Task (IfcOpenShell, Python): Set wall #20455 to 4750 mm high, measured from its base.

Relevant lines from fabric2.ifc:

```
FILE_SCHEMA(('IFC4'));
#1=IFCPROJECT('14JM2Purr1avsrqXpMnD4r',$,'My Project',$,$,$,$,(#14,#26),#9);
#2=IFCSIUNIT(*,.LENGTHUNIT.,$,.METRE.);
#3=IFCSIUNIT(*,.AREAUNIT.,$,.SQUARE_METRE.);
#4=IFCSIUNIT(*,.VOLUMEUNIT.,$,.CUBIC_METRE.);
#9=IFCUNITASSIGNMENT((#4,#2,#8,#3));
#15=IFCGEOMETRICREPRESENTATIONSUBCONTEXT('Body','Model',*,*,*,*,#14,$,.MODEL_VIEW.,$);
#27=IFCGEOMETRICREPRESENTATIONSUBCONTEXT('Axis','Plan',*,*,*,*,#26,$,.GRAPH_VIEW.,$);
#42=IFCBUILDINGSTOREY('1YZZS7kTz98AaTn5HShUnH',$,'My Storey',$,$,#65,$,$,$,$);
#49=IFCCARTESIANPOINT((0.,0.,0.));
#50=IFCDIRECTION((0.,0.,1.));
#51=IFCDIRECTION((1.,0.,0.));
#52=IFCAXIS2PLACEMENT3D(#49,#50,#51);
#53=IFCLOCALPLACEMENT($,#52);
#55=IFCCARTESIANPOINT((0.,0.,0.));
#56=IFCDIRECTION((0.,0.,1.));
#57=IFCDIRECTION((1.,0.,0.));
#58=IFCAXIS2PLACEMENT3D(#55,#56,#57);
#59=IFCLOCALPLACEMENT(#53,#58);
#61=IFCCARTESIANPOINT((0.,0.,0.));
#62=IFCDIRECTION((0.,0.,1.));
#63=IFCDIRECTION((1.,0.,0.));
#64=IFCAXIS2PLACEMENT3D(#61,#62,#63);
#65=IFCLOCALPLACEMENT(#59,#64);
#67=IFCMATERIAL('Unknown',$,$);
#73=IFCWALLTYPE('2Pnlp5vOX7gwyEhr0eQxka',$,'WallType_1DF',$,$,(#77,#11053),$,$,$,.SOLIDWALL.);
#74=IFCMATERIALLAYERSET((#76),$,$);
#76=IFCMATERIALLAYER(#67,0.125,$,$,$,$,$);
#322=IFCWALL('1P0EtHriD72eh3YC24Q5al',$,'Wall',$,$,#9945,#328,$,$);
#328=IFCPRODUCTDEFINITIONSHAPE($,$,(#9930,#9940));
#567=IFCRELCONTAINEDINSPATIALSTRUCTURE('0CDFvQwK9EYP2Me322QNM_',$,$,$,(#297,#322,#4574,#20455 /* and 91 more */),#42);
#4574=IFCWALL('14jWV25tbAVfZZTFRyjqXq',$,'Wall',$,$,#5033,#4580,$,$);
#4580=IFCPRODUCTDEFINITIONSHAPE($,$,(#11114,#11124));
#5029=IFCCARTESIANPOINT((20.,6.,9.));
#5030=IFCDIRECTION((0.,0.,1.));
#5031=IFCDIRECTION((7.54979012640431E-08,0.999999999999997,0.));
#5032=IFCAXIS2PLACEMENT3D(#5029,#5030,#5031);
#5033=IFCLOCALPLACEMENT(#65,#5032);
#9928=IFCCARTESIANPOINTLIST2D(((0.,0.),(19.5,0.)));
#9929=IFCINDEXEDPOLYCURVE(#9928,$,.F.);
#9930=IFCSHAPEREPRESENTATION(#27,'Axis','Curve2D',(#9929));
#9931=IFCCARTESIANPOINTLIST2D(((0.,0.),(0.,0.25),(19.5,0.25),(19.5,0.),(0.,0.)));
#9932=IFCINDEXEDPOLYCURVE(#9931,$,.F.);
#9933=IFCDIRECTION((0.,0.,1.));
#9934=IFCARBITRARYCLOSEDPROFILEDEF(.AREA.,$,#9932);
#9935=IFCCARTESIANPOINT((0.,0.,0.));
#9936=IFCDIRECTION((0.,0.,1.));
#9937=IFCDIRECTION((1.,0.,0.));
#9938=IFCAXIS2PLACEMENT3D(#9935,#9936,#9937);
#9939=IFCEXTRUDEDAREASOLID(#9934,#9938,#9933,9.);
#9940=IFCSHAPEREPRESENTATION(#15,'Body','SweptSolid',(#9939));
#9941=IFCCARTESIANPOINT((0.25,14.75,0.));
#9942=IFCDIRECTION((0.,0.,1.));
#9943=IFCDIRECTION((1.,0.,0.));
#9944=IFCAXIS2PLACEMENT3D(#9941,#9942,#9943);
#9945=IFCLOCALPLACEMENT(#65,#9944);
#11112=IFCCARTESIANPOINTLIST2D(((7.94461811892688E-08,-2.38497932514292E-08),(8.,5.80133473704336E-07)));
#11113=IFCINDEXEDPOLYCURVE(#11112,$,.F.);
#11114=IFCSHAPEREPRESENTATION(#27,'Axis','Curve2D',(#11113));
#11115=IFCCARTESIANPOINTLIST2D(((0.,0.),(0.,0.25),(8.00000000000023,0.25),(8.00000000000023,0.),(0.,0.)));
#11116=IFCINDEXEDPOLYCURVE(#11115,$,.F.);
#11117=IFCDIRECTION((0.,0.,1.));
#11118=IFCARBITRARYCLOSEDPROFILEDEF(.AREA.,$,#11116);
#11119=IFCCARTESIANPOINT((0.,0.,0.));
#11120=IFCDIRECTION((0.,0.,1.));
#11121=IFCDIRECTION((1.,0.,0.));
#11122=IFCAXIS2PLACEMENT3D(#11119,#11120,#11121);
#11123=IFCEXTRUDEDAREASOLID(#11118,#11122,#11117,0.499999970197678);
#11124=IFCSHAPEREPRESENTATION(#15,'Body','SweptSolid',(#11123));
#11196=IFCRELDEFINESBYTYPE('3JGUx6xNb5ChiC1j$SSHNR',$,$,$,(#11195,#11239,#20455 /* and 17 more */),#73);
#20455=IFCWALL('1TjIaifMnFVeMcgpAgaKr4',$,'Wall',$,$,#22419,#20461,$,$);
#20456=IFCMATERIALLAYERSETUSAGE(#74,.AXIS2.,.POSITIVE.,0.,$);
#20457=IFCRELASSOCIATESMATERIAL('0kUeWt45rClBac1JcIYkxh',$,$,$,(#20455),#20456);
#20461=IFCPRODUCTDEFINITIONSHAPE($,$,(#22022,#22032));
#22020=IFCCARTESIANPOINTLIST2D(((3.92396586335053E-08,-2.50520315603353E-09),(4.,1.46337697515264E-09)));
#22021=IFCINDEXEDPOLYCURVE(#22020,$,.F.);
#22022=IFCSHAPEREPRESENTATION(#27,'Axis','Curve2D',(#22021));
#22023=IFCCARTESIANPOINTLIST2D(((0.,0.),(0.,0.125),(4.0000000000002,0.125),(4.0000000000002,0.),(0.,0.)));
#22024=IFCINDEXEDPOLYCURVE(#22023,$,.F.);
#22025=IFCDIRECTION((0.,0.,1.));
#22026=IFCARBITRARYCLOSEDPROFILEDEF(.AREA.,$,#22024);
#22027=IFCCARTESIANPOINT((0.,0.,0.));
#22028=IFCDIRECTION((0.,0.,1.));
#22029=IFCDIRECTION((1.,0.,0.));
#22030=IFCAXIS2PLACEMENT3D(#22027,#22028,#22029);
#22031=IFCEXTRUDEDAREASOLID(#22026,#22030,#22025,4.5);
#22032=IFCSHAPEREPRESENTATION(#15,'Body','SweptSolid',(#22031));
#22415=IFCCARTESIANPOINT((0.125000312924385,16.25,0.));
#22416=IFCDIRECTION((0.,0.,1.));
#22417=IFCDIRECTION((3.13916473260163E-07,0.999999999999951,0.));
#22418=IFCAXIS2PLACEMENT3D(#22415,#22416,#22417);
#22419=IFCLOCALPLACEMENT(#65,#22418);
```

```python
import ifcopenshell
import ifcopenshell.geom
import ifcopenshell.util.representation
import ifcopenshell.util.shape

model = ifcopenshell.open("fabric2.ifc")
settings = ifcopenshell.geom.settings()


def volume(element):
    """Net volume in cubic metres, openings subtracted."""
    shape = ifcopenshell.geom.create_shape(settings, element)
    return ifcopenshell.util.shape.get_volume(shape.geometry)


wall = model.by_id(20455)
before = volume(wall)

body = ifcopenshell.util.representation.get_representation(wall, "Model", "Body")
solid = body.Items[0]
old_height = solid.Depth
solid.Depth = 4.75
after = volume(wall)

print(f"height {old_height:g} -> {solid.Depth:g}, volume {before:.3f} -> {after:.3f} m3")

model.write("fabric2_rev.ifc")
```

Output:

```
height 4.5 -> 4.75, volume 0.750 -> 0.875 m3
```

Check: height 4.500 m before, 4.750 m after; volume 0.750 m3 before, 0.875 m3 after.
